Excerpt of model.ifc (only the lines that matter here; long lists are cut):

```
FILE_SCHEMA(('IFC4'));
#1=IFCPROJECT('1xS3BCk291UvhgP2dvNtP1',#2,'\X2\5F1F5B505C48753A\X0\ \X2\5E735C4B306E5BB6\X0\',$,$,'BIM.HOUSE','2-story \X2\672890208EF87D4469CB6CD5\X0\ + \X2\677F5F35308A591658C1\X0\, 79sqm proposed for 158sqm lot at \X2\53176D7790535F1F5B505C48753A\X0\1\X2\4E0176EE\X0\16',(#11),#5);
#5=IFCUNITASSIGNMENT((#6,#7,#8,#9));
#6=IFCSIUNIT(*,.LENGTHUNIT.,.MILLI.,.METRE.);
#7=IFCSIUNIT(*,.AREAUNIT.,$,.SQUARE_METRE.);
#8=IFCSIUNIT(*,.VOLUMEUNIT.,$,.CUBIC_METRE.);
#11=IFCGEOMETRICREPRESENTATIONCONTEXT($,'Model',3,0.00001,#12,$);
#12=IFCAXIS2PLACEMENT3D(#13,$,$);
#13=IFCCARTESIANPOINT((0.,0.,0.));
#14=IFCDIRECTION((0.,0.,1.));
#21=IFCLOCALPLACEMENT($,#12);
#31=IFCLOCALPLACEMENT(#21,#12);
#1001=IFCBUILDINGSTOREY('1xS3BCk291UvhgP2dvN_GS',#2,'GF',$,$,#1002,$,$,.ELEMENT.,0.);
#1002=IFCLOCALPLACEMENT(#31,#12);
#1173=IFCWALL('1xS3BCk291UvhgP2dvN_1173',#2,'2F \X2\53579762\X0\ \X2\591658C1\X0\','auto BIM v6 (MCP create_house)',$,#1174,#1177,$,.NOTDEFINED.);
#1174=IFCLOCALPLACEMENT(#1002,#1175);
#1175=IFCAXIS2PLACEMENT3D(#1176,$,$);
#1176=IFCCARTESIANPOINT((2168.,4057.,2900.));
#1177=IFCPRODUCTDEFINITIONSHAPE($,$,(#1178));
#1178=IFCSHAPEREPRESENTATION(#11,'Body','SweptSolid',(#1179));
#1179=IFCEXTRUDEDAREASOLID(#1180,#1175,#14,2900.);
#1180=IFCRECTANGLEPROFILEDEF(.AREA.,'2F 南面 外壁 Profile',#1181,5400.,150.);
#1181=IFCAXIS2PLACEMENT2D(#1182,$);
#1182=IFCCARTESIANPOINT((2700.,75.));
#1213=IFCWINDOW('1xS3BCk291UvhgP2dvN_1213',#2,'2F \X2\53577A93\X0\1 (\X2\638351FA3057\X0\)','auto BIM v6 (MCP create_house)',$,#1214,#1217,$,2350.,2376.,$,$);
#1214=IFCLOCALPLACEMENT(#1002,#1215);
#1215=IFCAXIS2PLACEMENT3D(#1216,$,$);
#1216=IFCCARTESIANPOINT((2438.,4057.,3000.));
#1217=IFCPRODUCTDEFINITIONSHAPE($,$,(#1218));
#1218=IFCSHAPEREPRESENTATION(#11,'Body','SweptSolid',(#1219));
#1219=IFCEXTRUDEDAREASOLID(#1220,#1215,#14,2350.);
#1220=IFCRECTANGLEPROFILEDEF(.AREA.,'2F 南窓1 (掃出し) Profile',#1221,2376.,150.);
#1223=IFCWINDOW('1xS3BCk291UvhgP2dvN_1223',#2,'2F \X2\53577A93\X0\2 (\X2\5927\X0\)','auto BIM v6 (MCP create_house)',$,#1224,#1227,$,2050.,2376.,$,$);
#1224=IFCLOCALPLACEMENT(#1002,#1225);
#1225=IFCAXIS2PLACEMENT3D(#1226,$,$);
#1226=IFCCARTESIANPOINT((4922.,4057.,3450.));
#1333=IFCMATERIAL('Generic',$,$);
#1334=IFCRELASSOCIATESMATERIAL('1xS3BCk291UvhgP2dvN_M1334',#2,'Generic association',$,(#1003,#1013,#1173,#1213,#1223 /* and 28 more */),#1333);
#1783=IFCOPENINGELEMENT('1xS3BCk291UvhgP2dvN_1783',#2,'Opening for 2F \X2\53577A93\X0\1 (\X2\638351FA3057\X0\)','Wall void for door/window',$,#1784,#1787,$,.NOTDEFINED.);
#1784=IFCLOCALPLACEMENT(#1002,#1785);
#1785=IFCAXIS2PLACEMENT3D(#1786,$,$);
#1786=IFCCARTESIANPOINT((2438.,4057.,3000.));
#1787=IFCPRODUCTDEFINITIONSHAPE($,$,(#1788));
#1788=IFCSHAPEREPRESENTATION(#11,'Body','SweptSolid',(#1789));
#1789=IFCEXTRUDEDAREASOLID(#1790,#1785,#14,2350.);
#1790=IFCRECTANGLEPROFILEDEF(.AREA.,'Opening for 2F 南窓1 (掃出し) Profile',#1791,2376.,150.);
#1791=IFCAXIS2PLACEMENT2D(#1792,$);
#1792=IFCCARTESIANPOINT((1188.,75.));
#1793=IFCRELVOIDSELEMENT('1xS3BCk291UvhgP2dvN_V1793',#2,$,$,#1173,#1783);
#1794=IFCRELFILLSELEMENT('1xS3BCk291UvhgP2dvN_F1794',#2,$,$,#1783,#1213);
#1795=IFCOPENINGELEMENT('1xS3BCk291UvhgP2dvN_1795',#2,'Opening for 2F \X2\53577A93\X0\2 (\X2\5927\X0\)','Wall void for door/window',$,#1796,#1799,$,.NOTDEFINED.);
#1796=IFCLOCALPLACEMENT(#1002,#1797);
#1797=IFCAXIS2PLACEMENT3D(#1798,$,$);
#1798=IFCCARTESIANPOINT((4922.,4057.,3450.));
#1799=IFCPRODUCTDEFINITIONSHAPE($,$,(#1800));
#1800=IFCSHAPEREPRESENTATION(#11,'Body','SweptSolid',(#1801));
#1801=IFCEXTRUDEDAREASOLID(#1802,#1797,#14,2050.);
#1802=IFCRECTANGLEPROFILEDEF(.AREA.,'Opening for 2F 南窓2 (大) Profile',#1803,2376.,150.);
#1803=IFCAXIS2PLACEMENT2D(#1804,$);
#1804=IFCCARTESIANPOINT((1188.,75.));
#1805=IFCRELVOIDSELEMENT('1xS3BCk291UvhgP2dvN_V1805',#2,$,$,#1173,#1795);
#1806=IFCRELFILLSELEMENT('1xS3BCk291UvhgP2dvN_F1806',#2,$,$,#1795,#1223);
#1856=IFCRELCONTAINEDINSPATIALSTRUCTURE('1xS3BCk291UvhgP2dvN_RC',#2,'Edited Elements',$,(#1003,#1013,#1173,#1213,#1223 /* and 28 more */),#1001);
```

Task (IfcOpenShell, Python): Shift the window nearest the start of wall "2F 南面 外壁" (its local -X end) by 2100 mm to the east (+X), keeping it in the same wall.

```python
import ifcopenshell
import ifcopenshell.api.geometry
import ifcopenshell.util.placement

model = ifcopenshell.open("model.ifc")

window = model.by_guid("1xS3BCk291UvhgP2dvN_1213")
opening = window.FillsVoids[0].RelatingOpeningElement
wall = opening.VoidsElements[0].RelatingBuildingElement

wall_matrix = ifcopenshell.util.placement.get_local_placement(wall.ObjectPlacement)
shift = wall_matrix[:3, 0] * 2100.0
before = ifcopenshell.util.placement.get_local_placement(window.ObjectPlacement)[:3, 3].copy()

# The window is not placed relative to its opening, so move both.
for product in (opening, window):
    matrix = ifcopenshell.util.placement.get_local_placement(product.ObjectPlacement)
    matrix[:3, 3] += shift
    ifcopenshell.api.geometry.edit_object_placement(model, product=product, matrix=matrix, is_si=False)

after = ifcopenshell.util.placement.get_local_placement(window.ObjectPlacement)[:3, 3]
print("window moved by", (after - before).round(3) + 0.0)

model.write("model_updated.ifc")
```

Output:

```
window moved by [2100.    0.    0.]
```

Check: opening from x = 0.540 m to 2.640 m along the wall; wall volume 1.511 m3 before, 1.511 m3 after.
